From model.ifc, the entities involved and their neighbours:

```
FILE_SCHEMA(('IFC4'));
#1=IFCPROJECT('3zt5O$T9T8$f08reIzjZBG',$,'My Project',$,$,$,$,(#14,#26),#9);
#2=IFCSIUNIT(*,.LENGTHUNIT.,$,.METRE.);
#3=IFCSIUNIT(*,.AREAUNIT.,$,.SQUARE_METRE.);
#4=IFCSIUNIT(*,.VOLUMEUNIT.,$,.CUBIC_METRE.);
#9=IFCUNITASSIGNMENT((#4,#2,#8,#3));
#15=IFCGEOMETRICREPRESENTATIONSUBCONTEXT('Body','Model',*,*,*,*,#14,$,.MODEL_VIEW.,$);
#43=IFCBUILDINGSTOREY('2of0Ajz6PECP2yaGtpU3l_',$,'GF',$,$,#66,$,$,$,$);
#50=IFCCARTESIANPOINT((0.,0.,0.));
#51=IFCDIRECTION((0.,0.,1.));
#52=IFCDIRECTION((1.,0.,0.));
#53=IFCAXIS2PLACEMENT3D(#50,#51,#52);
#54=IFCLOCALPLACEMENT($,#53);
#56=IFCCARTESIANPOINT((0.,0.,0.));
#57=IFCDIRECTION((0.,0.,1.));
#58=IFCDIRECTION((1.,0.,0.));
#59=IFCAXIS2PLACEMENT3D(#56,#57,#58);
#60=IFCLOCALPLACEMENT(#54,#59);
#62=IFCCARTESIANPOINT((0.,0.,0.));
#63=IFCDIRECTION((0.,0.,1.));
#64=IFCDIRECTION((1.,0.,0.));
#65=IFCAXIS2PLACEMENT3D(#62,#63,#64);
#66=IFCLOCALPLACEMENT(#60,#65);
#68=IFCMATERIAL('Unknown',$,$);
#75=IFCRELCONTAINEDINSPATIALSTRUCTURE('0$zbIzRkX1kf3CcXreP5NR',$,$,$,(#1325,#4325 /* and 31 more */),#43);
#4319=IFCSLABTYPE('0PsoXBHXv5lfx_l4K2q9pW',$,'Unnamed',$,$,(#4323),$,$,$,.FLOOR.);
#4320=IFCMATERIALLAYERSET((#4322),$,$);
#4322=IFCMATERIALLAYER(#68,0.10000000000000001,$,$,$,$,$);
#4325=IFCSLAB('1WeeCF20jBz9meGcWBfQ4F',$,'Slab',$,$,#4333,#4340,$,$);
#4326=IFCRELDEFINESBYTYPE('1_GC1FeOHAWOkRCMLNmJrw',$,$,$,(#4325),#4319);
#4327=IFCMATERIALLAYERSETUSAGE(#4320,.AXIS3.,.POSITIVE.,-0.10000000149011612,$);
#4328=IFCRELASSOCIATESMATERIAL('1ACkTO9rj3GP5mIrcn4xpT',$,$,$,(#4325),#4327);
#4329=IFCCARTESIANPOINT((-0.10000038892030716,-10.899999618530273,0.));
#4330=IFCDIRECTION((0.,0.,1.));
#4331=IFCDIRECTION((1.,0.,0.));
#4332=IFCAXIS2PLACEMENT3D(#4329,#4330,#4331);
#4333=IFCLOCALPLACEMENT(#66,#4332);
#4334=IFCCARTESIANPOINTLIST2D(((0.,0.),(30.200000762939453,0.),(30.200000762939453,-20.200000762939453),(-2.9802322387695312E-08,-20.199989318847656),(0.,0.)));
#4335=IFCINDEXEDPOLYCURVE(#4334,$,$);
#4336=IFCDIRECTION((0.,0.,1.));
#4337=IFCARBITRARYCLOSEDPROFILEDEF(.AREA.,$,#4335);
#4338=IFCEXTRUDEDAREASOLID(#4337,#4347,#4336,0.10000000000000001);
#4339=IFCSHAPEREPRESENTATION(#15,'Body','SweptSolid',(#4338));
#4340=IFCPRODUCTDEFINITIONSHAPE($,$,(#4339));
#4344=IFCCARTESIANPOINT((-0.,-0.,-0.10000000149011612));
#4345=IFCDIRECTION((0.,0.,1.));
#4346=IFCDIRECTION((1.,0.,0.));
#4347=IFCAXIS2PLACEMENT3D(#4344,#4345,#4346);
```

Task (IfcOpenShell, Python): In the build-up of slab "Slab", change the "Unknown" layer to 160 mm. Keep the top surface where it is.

```python
import ifcopenshell
import ifcopenshell.util.element
import ifcopenshell.util.representation
import ifcopenshell.util.unit

model = ifcopenshell.open("model.ifc")
unit_scale = ifcopenshell.util.unit.calculate_unit_scale(model)

layer_set = model.by_id(4320)
layer = next(l for l in layer_set.MaterialLayers if l.Material and l.Material.Name == "Unknown")
change = 0.16 / unit_scale - layer.LayerThickness
layer.LayerThickness += change

# Geometry does not follow the layer set by itself.
slabs = [e for e in ifcopenshell.util.element.get_elements_by_material(model, layer_set) if e.is_a("IfcSlab")]
for slab in sorted(slabs, key=lambda e: e.id()):
    body = ifcopenshell.util.representation.get_representation(slab, "Model", "Body")
    solid = body.Items[0]
    old_depth = solid.Depth
    solid.Depth += change
    # Extruded upwards: lower the start of the extrusion so the top stays.
    x, y, z = solid.Position.Location.Coordinates
    solid.Position.Location = model.createIfcCartesianPoint((x, y, z - change))
    print(slab.id(), f"{old_depth:g} -> {solid.Depth:g}")

# The layers are counted up from the underside, which has moved.
for usage in {ifcopenshell.util.element.get_material(slab) for slab in slabs}:
    usage.OffsetFromReferenceLine -= change

model.write("model-out.ifc")
```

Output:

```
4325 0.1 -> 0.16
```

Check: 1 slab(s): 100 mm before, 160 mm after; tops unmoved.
